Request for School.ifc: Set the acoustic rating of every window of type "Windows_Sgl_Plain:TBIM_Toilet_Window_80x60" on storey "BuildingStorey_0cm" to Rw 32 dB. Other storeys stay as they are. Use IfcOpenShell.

First a look at what the model holds.

```python
import ifcopenshell
import ifcopenshell.util.element

model = ifcopenshell.open("School.ifc")
print(model.schema)
storey = next(s for s in model.by_type("IfcBuildingStorey") if s.Name == "BuildingStorey_0cm")
windows = [e for e in ifcopenshell.util.element.get_decomposition(storey) if e.is_a("IfcWindow")]
seen = {}
for e in windows:
    element_type = ifcopenshell.util.element.get_type(e)
    key = (element_type.Name if element_type != e and element_type else None, ifcopenshell.util.element.get_pset(e, "Pset_WindowCommon", "AcousticRating"))
    seen[key] = seen.get(key, 0) + 1
for (name, value), count in sorted(seen.items(), key=str):
    print(count, "x", name, "|", value)
```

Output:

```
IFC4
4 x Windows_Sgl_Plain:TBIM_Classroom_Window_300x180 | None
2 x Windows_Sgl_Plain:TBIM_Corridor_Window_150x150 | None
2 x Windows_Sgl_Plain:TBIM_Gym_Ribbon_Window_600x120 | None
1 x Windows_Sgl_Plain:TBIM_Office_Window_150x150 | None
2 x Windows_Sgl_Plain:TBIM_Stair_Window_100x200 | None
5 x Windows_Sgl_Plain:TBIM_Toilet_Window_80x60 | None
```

```python
import ifcopenshell
import ifcopenshell.api.pset
import ifcopenshell.util.element

model = ifcopenshell.open("School.ifc")

storey = next(s for s in model.by_type("IfcBuildingStorey") if s.Name == "BuildingStorey_0cm")
windows = [e for e in ifcopenshell.util.element.get_decomposition(storey) if e.is_a("IfcWindow")]

count = 0
for e in windows:
    element_type = ifcopenshell.util.element.get_type(e)
    if element_type in (None, e) or element_type.Name != "Windows_Sgl_Plain:TBIM_Toilet_Window_80x60":
        continue
    # add_pset returns the element's existing set when there is one.
    pset = ifcopenshell.api.pset.add_pset(model, product=e, name="Pset_WindowCommon")
    ifcopenshell.api.pset.edit_pset(model, pset=pset, properties={"AcousticRating": "Rw 32 dB"})
    count += 1

print(count, "windows updated")

model.write("School_edited.ifc")
```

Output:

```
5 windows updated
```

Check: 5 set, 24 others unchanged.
